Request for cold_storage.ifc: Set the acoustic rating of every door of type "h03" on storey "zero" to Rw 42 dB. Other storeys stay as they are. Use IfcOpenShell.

First a look at what the model holds.

```python
import ifcopenshell
import ifcopenshell.util.element

model = ifcopenshell.open("cold_storage.ifc")
print(model.schema)
storey = next(s for s in model.by_type("IfcBuildingStorey") if s.Name == "zero")
doors = [e for e in ifcopenshell.util.element.get_decomposition(storey) if e.is_a("IfcDoor")]
seen = {}
for e in doors:
    element_type = ifcopenshell.util.element.get_type(e)
    key = (element_type.Name if element_type != e and element_type else None, ifcopenshell.util.element.get_pset(e, "Pset_DoorCommon", "AcousticRating"))
    seen[key] = seen.get(key, 0) + 1
for (name, value), count in sorted(seen.items(), key=str):
    print(count, "x", name, "|", value)
```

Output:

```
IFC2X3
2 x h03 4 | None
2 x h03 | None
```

```python
import ifcopenshell
import ifcopenshell.api.pset
import ifcopenshell.util.element

model = ifcopenshell.open("cold_storage.ifc")

storey = next(s for s in model.by_type("IfcBuildingStorey") if s.Name == "zero")
doors = [e for e in ifcopenshell.util.element.get_decomposition(storey) if e.is_a("IfcDoor")]

count = 0
for e in doors:
    element_type = ifcopenshell.util.element.get_type(e)
    if element_type in (None, e) or element_type.Name != "h03":
        continue
    # add_pset returns the element's existing set when there is one.
    pset = ifcopenshell.api.pset.add_pset(model, product=e, name="Pset_DoorCommon")
    ifcopenshell.api.pset.edit_pset(model, pset=pset, properties={"AcousticRating": "Rw 42 dB"})
    count += 1

print(count, "doors updated")

model.write("cold_storage_rev.ifc")
```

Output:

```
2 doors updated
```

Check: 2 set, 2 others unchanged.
